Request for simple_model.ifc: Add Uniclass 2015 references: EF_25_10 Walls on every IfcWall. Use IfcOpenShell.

First a look at what the model holds.

```python
import ifcopenshell

model = ifcopenshell.open("simple_model.ifc")
print(model.schema)
print("classifications:", [c.Name for c in model.by_type("IfcClassification")])
for ifc_class in ("IfcDoor", "IfcRoof", "IfcStair", "IfcWall", "IfcWindow"):
    print(ifc_class, len(model.by_type(ifc_class)))
```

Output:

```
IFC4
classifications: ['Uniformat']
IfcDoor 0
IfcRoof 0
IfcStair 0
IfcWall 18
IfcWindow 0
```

```python
import ifcopenshell
import ifcopenshell.api.classification

model = ifcopenshell.open("simple_model.ifc")

system = ifcopenshell.api.classification.add_classification(model, classification="Uniclass 2015")

codes = {
    "IfcWall": ("EF_25_10", "Walls"),
}
for ifc_class, (code, name) in codes.items():
    products = model.by_type(ifc_class)
    ifcopenshell.api.classification.add_reference(
        model, products=products, classification=system, identification=code, name=name
    )
    print(code, len(products))

model.write("simple_model-out.ifc")
```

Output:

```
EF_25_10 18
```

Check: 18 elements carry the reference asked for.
